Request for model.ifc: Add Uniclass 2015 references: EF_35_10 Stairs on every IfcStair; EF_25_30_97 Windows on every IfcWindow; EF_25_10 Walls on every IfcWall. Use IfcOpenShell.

First a look at what the model holds.

```python
import ifcopenshell

model = ifcopenshell.open("model.ifc")
print(model.schema)
print("classifications:", [c.Name for c in model.by_type("IfcClassification")])
for ifc_class in ("IfcDoor", "IfcRoof", "IfcStair", "IfcWall", "IfcWindow"):
    print(ifc_class, len(model.by_type(ifc_class)))
```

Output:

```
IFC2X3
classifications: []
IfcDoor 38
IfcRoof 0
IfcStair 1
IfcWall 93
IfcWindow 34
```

```python
import ifcopenshell
import ifcopenshell.api.classification

model = ifcopenshell.open("model.ifc")

# IFC2X3 requires Source and Edition and has no link from the project to the system.
system = model.create_entity("IfcClassification", Source="NBS", Edition="2015", Name="Uniclass 2015")

codes = {
    "IfcStair": ("EF_35_10", "Stairs"),
    "IfcWindow": ("EF_25_30_97", "Windows"),
    "IfcWall": ("EF_25_10", "Walls"),
}
for ifc_class, (code, name) in codes.items():
    products = model.by_type(ifc_class)
    ifcopenshell.api.classification.add_reference(
        model, products=products, classification=system, identification=code, name=name
    )
    print(code, len(products))

model.write("model-out.ifc")
```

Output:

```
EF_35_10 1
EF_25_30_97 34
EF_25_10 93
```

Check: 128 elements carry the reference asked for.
